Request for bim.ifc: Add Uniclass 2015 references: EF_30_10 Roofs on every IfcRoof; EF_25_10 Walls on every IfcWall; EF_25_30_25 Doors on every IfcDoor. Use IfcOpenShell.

First a look at what the model holds.

```python
import ifcopenshell

model = ifcopenshell.open("bim.ifc")
print(model.schema)
print("classifications:", [c.Name for c in model.by_type("IfcClassification")])
for ifc_class in ("IfcDoor", "IfcRoof", "IfcStair", "IfcWall", "IfcWindow"):
    print(ifc_class, len(model.by_type(ifc_class)))
```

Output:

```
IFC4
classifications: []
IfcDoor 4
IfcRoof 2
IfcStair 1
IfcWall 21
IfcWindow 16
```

```python
import ifcopenshell
import ifcopenshell.api.classification

model = ifcopenshell.open("bim.ifc")

system = ifcopenshell.api.classification.add_classification(model, classification="Uniclass 2015")

codes = {
    "IfcRoof": ("EF_30_10", "Roofs"),
    "IfcWall": ("EF_25_10", "Walls"),
    "IfcDoor": ("EF_25_30_25", "Doors"),
}
for ifc_class, (code, name) in codes.items():
    products = model.by_type(ifc_class)
    ifcopenshell.api.classification.add_reference(
        model, products=products, classification=system, identification=code, name=name
    )
    print(code, len(products))

model.write("bim_rev.ifc")
```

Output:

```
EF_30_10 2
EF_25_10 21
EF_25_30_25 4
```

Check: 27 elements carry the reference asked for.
